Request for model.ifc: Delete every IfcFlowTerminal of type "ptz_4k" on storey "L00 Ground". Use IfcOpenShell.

First a look at what the model holds.

```python
import ifcopenshell
import ifcopenshell.util.element

model = ifcopenshell.open("model.ifc")
print(model.schema)
storey = next(s for s in model.by_type("IfcBuildingStorey") if s.Name == "L00 Ground")
terminals = [e for e in ifcopenshell.util.element.get_decomposition(storey) if e.is_a("IfcFlowTerminal")]
seen = {}
for e in terminals:
    element_type = ifcopenshell.util.element.get_type(e)
    name = element_type.Name if element_type not in (None, e) else None
    seen[name] = seen.get(name, 0) + 1
for name, count in sorted(seen.items(), key=str):
    print(count, "x", name)
```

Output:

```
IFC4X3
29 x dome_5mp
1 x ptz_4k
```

```python
import ifcopenshell
import ifcopenshell.api.root
import ifcopenshell.util.element

model = ifcopenshell.open("model.ifc")

storey = next(s for s in model.by_type("IfcBuildingStorey") if s.Name == "L00 Ground")
terminals = [e for e in ifcopenshell.util.element.get_decomposition(storey) if e.is_a("IfcFlowTerminal")]
targets = [e for e in terminals if (t := ifcopenshell.util.element.get_type(e)) not in (None, e) and t.Name == "ptz_4k"]

for e in targets:
    ifcopenshell.api.root.remove_product(model, product=e)
print(len(targets), "removed")

model.write("model_rev.ifc")
```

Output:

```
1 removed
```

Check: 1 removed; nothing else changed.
